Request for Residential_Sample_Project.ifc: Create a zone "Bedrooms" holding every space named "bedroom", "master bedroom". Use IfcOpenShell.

First a look at what the model holds.

```python
import ifcopenshell

model = ifcopenshell.open("Residential_Sample_Project.ifc")
print(model.schema)
seen = {}
for space in model.by_type("IfcSpace"):
    seen[space.LongName] = seen.get(space.LongName, 0) + 1
for name, count in sorted(seen.items(), key=str):
    print(count, "x", name)
print("zones:", [z.Name for z in model.by_type("IfcZone")][:20])
```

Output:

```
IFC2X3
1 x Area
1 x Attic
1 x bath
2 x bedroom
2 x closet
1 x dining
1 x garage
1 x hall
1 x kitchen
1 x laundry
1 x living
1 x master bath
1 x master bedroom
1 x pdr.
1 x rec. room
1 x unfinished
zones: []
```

```python
import ifcopenshell
import ifcopenshell.api.group
import ifcopenshell.api.root

model = ifcopenshell.open("Residential_Sample_Project.ifc")

names = {"bedroom", "master bedroom"}
spaces = [s for s in model.by_type("IfcSpace") if s.LongName in names]

zone = ifcopenshell.api.root.create_entity(model, ifc_class="IfcZone", name="Bedrooms")
ifcopenshell.api.group.assign_group(model, products=spaces, group=zone)
print(len(spaces), "spaces in", zone.Name)

model.write("Residential_Sample_Project_updated.ifc")
```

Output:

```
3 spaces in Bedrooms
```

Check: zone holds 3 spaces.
